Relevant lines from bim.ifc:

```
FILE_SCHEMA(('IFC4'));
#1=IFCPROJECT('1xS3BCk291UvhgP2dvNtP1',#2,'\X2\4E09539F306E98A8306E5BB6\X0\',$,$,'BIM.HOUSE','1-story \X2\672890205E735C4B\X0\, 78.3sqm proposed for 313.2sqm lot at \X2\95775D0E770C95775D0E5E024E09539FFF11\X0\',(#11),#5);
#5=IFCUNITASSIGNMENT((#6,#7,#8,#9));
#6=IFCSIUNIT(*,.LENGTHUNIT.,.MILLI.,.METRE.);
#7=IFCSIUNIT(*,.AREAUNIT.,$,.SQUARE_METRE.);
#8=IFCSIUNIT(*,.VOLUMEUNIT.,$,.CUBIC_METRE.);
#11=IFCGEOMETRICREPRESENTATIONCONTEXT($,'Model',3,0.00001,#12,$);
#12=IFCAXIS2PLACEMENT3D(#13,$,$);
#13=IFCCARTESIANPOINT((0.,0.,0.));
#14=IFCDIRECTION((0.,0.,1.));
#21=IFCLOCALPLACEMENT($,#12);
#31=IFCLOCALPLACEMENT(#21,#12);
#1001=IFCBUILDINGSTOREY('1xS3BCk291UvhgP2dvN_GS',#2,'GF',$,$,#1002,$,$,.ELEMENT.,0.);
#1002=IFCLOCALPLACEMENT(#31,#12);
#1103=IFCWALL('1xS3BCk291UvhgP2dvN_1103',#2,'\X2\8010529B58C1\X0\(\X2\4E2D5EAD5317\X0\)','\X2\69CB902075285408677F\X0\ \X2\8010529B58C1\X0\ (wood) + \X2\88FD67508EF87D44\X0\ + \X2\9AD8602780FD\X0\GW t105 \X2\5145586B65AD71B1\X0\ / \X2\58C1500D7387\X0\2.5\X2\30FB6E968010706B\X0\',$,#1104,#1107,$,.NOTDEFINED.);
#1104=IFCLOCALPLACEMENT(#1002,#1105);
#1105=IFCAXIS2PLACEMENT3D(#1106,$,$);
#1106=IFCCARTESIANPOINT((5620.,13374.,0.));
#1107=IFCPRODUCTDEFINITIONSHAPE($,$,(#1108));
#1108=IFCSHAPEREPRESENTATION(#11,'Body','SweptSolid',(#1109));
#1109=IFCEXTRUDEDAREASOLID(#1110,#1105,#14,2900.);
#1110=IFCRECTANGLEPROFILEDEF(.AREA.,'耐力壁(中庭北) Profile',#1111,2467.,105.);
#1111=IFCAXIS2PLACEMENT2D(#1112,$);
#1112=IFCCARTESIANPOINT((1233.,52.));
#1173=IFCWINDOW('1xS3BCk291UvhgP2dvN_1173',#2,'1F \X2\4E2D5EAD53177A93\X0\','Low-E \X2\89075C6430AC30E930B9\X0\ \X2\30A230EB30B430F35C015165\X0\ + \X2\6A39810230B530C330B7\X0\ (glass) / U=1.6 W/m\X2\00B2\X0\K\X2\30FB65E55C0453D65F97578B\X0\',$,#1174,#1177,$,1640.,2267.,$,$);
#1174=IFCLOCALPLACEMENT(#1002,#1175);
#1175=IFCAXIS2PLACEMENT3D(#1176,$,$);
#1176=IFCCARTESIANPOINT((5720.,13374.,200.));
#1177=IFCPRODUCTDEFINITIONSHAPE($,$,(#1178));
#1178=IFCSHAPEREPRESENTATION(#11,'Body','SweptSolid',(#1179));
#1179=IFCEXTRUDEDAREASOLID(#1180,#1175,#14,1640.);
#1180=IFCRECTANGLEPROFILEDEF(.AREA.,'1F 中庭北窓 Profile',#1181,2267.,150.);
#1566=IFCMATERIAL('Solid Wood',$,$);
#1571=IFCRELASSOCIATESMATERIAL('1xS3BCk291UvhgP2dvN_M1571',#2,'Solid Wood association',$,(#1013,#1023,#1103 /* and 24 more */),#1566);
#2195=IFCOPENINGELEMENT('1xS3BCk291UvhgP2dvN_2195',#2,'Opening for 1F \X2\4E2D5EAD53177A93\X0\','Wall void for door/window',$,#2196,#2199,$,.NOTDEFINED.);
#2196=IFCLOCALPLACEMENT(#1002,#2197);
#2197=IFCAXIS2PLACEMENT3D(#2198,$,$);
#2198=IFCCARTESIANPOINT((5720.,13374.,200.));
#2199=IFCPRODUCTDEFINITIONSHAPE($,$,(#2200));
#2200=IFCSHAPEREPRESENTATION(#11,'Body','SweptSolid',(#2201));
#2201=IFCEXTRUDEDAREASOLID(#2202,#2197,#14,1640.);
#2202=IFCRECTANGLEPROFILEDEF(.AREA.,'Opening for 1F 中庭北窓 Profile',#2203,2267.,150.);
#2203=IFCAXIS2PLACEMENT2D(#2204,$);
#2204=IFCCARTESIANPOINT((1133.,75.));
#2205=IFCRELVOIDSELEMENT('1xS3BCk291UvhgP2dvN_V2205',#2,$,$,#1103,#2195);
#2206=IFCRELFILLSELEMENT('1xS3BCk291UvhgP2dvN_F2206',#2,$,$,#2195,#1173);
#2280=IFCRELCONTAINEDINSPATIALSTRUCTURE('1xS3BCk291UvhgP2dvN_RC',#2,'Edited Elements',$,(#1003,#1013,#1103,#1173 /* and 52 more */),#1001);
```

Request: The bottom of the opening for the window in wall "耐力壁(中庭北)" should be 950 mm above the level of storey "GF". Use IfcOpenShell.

```python
import numpy as np
import ifcopenshell
import ifcopenshell.api.geometry
import ifcopenshell.geom
import ifcopenshell.util.element
import ifcopenshell.util.placement
import ifcopenshell.util.shape
import ifcopenshell.util.unit

model = ifcopenshell.open("bim.ifc")
unit_scale = ifcopenshell.util.unit.calculate_unit_scale(model)

window = model.by_guid("1xS3BCk291UvhgP2dvN_1173")
opening = window.FillsVoids[0].RelatingOpeningElement
storey = ifcopenshell.util.element.get_container(window, ifc_class="IfcBuildingStorey")
level = ifcopenshell.util.placement.get_local_placement(storey.ObjectPlacement)[2, 3]

# The opening's origin need not be at the sill, so measure its lowest point.
shape = ifcopenshell.geom.create_shape(ifcopenshell.geom.settings(), opening)
bottom = ifcopenshell.util.shape.get_shape_bottom_elevation(shape, shape.geometry) / unit_scale
dz = level + 0.95 / unit_scale - bottom

shift = np.array([0.0, 0.0, dz])
# The window is not placed relative to its opening, so move both.
for product in (opening, window):
    matrix = ifcopenshell.util.placement.get_local_placement(product.ObjectPlacement)
    matrix[:3, 3] += shift
    ifcopenshell.api.geometry.edit_object_placement(model, product=product, matrix=matrix, is_si=False)

print(f"moved by {dz * unit_scale:+.3f} m")

model.write("bim_updated.ifc")
```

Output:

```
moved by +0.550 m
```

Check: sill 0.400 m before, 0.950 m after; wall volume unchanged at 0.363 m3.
